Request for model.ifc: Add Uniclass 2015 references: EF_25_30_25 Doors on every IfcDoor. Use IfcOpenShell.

First a look at what the model holds.

```python
import ifcopenshell

model = ifcopenshell.open("model.ifc")
print(model.schema)
print("classifications:", [c.Name for c in model.by_type("IfcClassification")])
for ifc_class in ("IfcDoor", "IfcRoof", "IfcStair", "IfcWall", "IfcWindow"):
    print(ifc_class, len(model.by_type(ifc_class)))
```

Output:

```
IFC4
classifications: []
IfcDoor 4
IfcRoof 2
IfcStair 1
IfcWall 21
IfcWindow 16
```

```python
import ifcopenshell
import ifcopenshell.api.classification

model = ifcopenshell.open("model.ifc")

system = ifcopenshell.api.classification.add_classification(model, classification="Uniclass 2015")

codes = {
    "IfcDoor": ("EF_25_30_25", "Doors"),
}
for ifc_class, (code, name) in codes.items():
    products = model.by_type(ifc_class)
    ifcopenshell.api.classification.add_reference(
        model, products=products, classification=system, identification=code, name=name
    )
    print(code, len(products))

model.write("model_updated.ifc")
```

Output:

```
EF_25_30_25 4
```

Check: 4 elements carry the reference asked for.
